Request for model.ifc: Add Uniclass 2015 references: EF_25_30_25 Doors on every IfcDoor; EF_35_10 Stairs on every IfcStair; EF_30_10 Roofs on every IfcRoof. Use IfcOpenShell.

First a look at what the model holds.

```python
import ifcopenshell

model = ifcopenshell.open("model.ifc")
print(model.schema)
print("classifications:", [c.Name for c in model.by_type("IfcClassification")])
for ifc_class in ("IfcDoor", "IfcRoof", "IfcStair", "IfcWall", "IfcWindow"):
    print(ifc_class, len(model.by_type(ifc_class)))
```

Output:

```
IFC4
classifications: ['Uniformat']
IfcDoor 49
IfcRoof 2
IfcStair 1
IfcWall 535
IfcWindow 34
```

```python
import ifcopenshell
import ifcopenshell.api.classification

model = ifcopenshell.open("model.ifc")

system = ifcopenshell.api.classification.add_classification(model, classification="Uniclass 2015")

codes = {
    "IfcDoor": ("EF_25_30_25", "Doors"),
    "IfcStair": ("EF_35_10", "Stairs"),
    "IfcRoof": ("EF_30_10", "Roofs"),
}
for ifc_class, (code, name) in codes.items():
    products = model.by_type(ifc_class)
    ifcopenshell.api.classification.add_reference(
        model, products=products, classification=system, identification=code, name=name
    )
    print(code, len(products))

model.write("model_v2.ifc")
```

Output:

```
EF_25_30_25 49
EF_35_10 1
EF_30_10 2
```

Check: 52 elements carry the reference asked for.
